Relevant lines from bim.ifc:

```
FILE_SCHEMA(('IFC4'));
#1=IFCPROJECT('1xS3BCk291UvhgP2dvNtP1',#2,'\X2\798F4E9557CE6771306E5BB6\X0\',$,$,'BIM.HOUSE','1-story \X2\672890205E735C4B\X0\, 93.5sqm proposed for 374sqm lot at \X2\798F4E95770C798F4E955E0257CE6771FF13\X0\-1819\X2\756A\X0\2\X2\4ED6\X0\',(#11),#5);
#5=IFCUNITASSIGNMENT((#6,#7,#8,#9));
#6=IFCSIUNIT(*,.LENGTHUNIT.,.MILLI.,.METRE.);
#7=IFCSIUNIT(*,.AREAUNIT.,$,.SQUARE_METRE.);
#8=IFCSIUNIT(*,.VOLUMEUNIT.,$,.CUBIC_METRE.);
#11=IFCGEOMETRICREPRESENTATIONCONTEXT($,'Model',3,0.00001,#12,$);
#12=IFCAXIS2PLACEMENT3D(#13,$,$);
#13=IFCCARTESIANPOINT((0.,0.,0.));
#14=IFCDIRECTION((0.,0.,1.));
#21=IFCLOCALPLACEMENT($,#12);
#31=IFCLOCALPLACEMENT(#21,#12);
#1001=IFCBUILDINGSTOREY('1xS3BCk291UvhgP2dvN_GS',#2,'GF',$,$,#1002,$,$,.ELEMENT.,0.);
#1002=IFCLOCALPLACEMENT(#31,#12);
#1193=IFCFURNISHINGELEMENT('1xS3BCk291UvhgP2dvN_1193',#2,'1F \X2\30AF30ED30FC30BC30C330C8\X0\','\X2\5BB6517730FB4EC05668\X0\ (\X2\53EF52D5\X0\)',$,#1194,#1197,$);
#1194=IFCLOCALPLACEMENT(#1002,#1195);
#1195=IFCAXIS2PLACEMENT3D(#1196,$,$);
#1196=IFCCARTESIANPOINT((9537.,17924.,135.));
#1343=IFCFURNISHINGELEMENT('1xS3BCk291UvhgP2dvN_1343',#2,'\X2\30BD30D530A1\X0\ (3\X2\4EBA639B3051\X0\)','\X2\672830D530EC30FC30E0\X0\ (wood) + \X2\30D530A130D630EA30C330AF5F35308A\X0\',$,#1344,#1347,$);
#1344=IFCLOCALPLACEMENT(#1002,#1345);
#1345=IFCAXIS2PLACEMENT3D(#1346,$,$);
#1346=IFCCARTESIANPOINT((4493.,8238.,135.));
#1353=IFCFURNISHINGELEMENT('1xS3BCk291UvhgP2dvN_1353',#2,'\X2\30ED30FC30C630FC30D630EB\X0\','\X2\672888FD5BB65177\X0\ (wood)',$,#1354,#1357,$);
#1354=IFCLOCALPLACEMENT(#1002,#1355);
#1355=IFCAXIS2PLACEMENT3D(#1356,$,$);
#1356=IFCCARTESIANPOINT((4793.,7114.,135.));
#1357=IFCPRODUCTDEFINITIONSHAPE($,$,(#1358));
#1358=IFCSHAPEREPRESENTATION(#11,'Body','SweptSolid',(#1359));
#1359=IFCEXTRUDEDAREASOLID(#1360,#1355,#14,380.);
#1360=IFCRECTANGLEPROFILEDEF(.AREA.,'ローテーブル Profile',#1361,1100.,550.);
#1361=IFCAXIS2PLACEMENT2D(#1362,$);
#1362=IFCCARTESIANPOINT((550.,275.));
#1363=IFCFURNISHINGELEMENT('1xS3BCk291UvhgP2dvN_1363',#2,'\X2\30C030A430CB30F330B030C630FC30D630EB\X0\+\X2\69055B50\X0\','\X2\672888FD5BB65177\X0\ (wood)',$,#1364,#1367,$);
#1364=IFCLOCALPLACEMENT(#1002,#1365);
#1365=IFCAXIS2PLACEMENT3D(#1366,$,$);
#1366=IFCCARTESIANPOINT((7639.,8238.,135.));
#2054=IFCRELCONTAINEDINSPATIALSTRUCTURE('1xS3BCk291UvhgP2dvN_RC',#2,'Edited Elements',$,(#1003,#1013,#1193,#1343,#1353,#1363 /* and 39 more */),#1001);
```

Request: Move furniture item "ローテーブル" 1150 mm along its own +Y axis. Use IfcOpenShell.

```python
import ifcopenshell
import ifcopenshell.api.geometry
import ifcopenshell.util.placement

model = ifcopenshell.open("bim.ifc")

item = model.by_guid("1xS3BCk291UvhgP2dvN_1353")
matrix = ifcopenshell.util.placement.get_local_placement(item.ObjectPlacement)
matrix[:3, 3] += matrix[:3, 1] * 1150.0
ifcopenshell.api.geometry.edit_object_placement(model, product=item, matrix=matrix, is_si=False)

print(ifcopenshell.util.placement.get_local_placement(item.ObjectPlacement).round(3) + 0.0)

model.write("bim_updated.ifc")
```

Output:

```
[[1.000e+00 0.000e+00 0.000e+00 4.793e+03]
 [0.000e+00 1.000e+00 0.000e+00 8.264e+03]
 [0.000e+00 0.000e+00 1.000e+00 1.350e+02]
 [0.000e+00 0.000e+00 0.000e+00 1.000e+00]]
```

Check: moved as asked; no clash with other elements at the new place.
